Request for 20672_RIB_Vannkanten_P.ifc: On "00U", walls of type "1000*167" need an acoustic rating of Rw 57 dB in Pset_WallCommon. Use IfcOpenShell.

First a look at what the model holds.

```python
import ifcopenshell
import ifcopenshell.util.element

model = ifcopenshell.open("20672_RIB_Vannkanten_P.ifc")
print(model.schema)
storey = next(s for s in model.by_type("IfcBuildingStorey") if s.Name == "00U")
walls = [e for e in ifcopenshell.util.element.get_decomposition(storey) if e.is_a("IfcWall")]
seen = {}
for e in walls:
    element_type = ifcopenshell.util.element.get_type(e)
    key = (element_type.Name if element_type != e and element_type else None, ifcopenshell.util.element.get_pset(e, "Pset_WallCommon", "AcousticRating"))
    seen[key] = seen.get(key, 0) + 1
for (name, value), count in sorted(seen.items(), key=str):
    print(count, "x", name, "|", value)
```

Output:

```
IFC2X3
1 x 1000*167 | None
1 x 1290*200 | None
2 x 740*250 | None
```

```python
import ifcopenshell
import ifcopenshell.api.pset
import ifcopenshell.util.element

model = ifcopenshell.open("20672_RIB_Vannkanten_P.ifc")

storey = next(s for s in model.by_type("IfcBuildingStorey") if s.Name == "00U")
walls = [e for e in ifcopenshell.util.element.get_decomposition(storey) if e.is_a("IfcWall")]

count = 0
for e in walls:
    element_type = ifcopenshell.util.element.get_type(e)
    if element_type in (None, e) or element_type.Name != "1000*167":
        continue
    # add_pset returns the element's existing set when there is one.
    pset = ifcopenshell.api.pset.add_pset(model, product=e, name="Pset_WallCommon")
    ifcopenshell.api.pset.edit_pset(model, pset=pset, properties={"AcousticRating": "Rw 57 dB"})
    count += 1

print(count, "walls updated")

model.write("20672_RIB_Vannkanten_P_updated.ifc")
```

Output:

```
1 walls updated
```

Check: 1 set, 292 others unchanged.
